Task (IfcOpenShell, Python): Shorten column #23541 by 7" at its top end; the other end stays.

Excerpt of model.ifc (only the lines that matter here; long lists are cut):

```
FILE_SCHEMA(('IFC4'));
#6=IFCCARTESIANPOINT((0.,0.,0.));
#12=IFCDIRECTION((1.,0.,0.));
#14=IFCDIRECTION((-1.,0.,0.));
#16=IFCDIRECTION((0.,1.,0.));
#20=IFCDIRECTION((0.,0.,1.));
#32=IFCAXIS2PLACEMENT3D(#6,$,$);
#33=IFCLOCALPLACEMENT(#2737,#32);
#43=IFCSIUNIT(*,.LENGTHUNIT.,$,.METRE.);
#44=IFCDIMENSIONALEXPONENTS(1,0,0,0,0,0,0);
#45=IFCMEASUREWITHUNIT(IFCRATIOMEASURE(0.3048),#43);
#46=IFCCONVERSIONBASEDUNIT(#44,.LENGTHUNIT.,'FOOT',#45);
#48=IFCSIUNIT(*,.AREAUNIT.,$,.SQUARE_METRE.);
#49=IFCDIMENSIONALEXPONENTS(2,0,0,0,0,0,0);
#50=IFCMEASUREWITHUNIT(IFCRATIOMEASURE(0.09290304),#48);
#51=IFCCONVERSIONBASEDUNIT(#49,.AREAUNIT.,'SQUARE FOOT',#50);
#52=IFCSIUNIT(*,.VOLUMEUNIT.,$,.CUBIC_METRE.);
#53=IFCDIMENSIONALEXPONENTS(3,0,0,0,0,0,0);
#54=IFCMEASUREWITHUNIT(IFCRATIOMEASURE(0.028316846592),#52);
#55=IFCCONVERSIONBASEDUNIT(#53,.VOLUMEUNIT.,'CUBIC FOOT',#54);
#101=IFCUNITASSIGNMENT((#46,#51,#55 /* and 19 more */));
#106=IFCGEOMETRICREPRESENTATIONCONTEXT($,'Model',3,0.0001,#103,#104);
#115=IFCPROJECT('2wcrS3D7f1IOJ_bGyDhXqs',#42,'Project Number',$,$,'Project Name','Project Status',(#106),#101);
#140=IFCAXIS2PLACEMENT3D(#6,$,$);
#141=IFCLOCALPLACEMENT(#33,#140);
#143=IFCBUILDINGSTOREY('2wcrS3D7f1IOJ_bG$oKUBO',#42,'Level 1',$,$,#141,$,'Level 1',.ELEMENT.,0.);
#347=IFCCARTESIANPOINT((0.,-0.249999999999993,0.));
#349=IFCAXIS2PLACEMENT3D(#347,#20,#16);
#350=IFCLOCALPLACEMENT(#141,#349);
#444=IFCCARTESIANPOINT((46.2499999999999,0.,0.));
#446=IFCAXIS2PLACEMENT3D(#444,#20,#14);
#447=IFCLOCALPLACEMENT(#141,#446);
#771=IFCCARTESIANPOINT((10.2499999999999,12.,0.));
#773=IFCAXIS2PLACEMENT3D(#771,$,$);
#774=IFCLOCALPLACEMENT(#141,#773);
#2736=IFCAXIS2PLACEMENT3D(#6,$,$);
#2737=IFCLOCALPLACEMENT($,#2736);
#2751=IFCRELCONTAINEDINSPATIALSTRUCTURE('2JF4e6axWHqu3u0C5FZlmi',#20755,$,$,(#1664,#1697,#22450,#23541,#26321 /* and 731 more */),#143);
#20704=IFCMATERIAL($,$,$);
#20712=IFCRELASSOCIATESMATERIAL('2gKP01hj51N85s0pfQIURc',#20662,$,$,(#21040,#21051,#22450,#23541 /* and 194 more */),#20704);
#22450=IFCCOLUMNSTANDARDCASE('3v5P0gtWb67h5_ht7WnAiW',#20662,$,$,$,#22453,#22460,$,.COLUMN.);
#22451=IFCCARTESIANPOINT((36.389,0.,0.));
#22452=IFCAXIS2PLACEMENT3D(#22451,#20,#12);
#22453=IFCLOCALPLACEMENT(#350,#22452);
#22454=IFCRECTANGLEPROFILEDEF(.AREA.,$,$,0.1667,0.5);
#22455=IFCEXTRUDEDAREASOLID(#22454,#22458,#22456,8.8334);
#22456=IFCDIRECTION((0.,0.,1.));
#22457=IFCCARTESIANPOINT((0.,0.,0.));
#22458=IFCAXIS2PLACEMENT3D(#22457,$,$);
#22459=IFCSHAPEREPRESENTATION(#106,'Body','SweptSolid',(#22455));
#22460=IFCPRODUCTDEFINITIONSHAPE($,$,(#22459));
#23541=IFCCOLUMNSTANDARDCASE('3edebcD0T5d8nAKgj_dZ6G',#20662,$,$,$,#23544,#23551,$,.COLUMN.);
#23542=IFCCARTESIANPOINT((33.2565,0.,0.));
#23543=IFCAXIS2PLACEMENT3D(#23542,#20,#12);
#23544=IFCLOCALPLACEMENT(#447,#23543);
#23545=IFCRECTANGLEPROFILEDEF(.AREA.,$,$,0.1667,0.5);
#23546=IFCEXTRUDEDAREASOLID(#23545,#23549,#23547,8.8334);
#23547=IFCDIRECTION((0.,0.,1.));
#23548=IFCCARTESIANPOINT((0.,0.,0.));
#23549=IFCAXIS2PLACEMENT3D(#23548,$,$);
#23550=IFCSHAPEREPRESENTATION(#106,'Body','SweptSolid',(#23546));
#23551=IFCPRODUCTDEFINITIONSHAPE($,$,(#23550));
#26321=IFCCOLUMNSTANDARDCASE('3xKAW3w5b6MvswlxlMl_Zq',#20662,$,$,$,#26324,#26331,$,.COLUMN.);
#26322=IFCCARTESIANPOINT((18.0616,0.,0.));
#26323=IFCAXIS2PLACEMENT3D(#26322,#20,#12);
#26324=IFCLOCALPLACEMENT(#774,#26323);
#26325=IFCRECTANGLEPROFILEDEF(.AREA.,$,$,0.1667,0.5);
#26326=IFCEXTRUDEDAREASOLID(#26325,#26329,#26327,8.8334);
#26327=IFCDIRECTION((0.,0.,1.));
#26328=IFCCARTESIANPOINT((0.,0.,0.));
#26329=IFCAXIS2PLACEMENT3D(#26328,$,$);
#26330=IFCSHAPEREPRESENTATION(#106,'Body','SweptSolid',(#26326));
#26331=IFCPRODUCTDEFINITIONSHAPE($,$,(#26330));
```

```python
import ifcopenshell
import ifcopenshell.util.unit

model = ifcopenshell.open("model.ifc")
unit_scale = ifcopenshell.util.unit.calculate_unit_scale(model)

member = model.by_id(23541)
change = -7 * 0.0254 / unit_scale

# The extrusion runs towards the end named, so only its depth changes.
body = next(r for r in member.Representation.Representations if r.RepresentationIdentifier == "Body")
solid = body.Items[0]
old_length = solid.Depth
solid.Depth += change

print(f"length {old_length:g} -> {solid.Depth:g}")

model.write("model_edited.ifc")
```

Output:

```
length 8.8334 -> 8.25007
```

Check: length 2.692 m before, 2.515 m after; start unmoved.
